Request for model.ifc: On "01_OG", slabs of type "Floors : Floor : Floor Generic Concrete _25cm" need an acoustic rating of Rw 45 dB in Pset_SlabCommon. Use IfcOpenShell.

First a look at what the model holds.

```python
import ifcopenshell
import ifcopenshell.util.element

model = ifcopenshell.open("model.ifc")
print(model.schema)
storey = next(s for s in model.by_type("IfcBuildingStorey") if s.Name == "01_OG")
slabs = [e for e in ifcopenshell.util.element.get_decomposition(storey) if e.is_a("IfcSlab")]
seen = {}
for e in slabs:
    element_type = ifcopenshell.util.element.get_type(e)
    key = (element_type.Name if element_type != e and element_type else None, ifcopenshell.util.element.get_pset(e, "Pset_SlabCommon", "AcousticRating"))
    seen[key] = seen.get(key, 0) + 1
for (name, value), count in sorted(seen.items(), key=str):
    print(count, "x", name, "|", value)
```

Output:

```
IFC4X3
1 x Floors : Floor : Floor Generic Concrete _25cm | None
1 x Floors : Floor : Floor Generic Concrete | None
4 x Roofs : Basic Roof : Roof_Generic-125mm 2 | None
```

```python
import ifcopenshell
import ifcopenshell.api.pset
import ifcopenshell.util.element

model = ifcopenshell.open("model.ifc")

storey = next(s for s in model.by_type("IfcBuildingStorey") if s.Name == "01_OG")
slabs = [e for e in ifcopenshell.util.element.get_decomposition(storey) if e.is_a("IfcSlab")]

count = 0
for e in slabs:
    element_type = ifcopenshell.util.element.get_type(e)
    if element_type in (None, e) or element_type.Name != "Floors : Floor : Floor Generic Concrete _25cm":
        continue
    # add_pset returns the element's existing set when there is one.
    pset = ifcopenshell.api.pset.add_pset(model, product=e, name="Pset_SlabCommon")
    ifcopenshell.api.pset.edit_pset(model, pset=pset, properties={"AcousticRating": "Rw 45 dB"})
    count += 1

print(count, "slabs updated")

model.write("model_edited.ifc")
```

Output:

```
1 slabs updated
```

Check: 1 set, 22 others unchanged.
